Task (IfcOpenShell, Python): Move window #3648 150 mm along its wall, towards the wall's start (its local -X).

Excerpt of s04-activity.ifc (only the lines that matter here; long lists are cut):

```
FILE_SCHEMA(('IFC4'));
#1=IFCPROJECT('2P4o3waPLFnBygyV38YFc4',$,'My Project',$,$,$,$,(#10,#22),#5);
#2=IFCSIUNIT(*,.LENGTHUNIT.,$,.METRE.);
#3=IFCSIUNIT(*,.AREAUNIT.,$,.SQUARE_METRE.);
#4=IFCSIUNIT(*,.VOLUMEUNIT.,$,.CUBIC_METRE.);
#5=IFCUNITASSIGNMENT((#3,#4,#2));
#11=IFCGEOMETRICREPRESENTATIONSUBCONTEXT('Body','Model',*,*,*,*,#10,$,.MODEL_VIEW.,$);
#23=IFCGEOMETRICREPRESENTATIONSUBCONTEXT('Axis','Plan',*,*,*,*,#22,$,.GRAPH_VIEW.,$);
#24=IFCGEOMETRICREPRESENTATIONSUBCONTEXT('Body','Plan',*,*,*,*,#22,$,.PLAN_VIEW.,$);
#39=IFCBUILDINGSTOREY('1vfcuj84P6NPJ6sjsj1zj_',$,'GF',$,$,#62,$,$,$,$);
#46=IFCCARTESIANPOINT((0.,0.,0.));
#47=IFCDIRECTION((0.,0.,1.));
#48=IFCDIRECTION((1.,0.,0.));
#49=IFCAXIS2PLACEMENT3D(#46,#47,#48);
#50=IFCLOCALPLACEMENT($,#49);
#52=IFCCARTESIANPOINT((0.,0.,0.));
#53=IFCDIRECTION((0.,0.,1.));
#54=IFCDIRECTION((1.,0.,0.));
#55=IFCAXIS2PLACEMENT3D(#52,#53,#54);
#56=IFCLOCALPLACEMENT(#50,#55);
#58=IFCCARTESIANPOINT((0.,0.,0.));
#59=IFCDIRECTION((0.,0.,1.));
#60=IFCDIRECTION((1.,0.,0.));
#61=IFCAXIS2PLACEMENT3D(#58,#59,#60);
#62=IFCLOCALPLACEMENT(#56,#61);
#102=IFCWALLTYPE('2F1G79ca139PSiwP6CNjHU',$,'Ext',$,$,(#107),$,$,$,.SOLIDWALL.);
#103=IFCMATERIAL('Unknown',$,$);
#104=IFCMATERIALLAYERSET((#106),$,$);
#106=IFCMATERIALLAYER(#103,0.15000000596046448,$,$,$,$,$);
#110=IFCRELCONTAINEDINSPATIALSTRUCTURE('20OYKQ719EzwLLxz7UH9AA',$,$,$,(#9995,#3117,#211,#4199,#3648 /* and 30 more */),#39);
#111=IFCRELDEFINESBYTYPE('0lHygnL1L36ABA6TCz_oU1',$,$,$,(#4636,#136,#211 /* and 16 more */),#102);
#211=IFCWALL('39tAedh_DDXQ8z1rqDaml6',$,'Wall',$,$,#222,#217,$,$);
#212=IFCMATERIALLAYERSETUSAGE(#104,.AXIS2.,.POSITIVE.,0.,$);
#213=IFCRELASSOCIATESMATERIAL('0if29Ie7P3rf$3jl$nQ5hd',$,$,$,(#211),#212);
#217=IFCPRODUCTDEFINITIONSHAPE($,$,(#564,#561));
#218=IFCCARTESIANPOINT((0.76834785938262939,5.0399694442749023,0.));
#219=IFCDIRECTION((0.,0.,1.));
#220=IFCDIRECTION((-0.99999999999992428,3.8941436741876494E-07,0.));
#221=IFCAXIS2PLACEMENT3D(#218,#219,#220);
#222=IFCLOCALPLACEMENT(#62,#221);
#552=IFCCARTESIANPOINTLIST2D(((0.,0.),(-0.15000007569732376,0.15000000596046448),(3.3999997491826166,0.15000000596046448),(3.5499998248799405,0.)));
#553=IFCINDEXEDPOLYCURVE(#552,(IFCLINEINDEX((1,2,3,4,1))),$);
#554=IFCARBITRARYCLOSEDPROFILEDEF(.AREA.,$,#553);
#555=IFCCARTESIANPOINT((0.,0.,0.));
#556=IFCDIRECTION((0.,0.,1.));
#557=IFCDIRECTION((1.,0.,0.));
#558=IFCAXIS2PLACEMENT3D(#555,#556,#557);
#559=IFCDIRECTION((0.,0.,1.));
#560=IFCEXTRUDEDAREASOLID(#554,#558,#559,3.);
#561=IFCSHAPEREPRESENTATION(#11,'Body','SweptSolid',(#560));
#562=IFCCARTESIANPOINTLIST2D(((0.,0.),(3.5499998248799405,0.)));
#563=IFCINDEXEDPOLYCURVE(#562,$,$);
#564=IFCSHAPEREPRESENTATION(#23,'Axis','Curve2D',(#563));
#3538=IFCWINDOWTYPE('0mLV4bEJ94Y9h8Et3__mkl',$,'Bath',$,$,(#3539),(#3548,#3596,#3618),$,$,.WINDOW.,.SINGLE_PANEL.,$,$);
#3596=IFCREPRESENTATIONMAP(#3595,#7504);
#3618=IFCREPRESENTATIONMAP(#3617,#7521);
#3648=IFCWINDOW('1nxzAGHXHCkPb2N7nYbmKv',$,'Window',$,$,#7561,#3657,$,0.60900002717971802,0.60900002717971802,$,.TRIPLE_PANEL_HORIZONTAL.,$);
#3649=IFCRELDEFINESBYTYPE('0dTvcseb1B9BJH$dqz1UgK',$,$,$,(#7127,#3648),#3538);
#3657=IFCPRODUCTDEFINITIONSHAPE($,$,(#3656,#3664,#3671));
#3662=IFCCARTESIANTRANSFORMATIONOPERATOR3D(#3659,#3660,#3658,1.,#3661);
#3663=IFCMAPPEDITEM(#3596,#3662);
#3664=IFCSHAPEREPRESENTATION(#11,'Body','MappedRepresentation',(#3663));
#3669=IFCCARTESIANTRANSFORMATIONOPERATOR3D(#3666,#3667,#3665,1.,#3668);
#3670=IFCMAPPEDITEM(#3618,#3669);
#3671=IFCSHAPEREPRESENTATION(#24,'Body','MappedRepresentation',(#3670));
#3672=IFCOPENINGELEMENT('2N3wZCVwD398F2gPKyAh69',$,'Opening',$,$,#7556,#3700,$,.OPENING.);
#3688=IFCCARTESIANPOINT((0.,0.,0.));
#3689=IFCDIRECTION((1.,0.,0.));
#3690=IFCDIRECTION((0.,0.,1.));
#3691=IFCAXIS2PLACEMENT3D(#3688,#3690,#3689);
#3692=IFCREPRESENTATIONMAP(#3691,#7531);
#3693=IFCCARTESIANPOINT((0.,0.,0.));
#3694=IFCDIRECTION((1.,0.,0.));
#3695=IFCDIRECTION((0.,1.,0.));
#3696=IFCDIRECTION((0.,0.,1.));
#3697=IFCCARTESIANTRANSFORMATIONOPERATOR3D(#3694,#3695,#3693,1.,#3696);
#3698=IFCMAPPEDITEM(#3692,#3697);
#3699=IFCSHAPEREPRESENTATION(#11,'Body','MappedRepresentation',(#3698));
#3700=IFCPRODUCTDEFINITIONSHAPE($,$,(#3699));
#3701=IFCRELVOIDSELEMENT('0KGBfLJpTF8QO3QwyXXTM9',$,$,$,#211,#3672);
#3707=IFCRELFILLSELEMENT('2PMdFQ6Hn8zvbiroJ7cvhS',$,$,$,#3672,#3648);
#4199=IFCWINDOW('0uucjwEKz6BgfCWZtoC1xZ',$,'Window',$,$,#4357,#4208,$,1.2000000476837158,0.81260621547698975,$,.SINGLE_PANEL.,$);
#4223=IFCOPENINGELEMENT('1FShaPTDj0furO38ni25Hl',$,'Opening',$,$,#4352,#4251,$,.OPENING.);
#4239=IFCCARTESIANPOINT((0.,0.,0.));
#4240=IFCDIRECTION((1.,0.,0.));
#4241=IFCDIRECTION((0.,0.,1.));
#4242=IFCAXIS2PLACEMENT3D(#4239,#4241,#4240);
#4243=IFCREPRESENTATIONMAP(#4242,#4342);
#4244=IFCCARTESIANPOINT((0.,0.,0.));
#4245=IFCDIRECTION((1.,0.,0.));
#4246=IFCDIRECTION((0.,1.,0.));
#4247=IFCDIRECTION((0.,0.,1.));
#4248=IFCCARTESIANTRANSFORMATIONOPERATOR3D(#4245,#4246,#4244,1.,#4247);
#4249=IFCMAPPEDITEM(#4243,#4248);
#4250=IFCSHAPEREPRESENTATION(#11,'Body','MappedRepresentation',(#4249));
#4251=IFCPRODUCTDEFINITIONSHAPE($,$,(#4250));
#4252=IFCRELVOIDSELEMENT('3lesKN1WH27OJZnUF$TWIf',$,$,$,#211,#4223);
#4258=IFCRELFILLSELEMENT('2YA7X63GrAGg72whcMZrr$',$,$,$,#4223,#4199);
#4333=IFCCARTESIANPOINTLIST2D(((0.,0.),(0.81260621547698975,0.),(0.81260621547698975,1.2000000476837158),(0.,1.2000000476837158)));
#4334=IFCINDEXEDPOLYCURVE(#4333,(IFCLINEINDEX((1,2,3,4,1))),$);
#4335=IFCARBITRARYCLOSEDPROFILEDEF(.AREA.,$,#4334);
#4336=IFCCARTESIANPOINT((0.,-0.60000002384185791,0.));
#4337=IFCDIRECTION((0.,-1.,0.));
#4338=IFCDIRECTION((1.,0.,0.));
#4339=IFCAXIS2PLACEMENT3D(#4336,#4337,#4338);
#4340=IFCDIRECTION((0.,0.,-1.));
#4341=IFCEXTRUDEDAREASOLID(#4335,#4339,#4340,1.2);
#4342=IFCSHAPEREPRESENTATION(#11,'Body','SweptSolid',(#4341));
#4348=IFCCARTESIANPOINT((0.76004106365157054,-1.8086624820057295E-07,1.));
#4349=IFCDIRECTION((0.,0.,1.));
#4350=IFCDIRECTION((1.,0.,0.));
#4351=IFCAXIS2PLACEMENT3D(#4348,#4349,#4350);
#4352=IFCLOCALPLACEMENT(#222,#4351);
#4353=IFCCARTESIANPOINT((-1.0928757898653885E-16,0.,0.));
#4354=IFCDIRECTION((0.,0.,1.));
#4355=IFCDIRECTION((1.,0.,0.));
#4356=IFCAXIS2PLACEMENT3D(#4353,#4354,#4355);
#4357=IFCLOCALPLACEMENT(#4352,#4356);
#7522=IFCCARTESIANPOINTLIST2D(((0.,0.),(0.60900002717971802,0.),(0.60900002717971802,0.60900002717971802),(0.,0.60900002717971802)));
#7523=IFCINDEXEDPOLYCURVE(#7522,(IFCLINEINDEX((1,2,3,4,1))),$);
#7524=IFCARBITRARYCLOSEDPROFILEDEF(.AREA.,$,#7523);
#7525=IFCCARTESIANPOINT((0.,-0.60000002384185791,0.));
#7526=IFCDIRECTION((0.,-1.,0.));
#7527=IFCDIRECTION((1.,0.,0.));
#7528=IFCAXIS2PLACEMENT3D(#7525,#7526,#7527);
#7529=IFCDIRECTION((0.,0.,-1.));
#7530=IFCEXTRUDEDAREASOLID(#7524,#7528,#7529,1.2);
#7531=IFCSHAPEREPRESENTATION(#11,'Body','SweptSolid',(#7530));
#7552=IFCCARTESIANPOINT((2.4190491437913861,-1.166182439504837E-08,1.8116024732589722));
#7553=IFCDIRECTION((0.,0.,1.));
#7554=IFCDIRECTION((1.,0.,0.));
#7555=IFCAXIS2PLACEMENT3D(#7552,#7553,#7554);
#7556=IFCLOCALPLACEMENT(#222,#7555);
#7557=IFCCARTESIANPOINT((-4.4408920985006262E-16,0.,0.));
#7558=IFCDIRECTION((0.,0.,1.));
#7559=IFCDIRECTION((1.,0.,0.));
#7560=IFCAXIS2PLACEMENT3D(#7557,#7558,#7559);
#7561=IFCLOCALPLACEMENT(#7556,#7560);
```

```python
import ifcopenshell
import ifcopenshell.api.geometry
import ifcopenshell.util.placement

model = ifcopenshell.open("s04-activity.ifc")

window = model.by_guid("1nxzAGHXHCkPb2N7nYbmKv")
opening = window.FillsVoids[0].RelatingOpeningElement
wall = opening.VoidsElements[0].RelatingBuildingElement

wall_matrix = ifcopenshell.util.placement.get_local_placement(wall.ObjectPlacement)
shift = wall_matrix[:3, 0] * -0.15
before = ifcopenshell.util.placement.get_local_placement(window.ObjectPlacement)[:3, 3].copy()

# The window is placed relative to its opening, so it follows when the opening moves.
matrix = ifcopenshell.util.placement.get_local_placement(opening.ObjectPlacement)
matrix[:3, 3] += shift
ifcopenshell.api.geometry.edit_object_placement(
    model, product=opening, matrix=matrix, is_si=False, should_transform_children=True
)

after = ifcopenshell.util.placement.get_local_placement(window.ObjectPlacement)[:3, 3]
print("window moved by", (after - before).round(3) + 0.0)

model.write("s04-activity_updated.ifc")
```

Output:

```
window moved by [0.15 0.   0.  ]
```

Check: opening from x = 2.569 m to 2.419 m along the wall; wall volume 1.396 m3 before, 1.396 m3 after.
